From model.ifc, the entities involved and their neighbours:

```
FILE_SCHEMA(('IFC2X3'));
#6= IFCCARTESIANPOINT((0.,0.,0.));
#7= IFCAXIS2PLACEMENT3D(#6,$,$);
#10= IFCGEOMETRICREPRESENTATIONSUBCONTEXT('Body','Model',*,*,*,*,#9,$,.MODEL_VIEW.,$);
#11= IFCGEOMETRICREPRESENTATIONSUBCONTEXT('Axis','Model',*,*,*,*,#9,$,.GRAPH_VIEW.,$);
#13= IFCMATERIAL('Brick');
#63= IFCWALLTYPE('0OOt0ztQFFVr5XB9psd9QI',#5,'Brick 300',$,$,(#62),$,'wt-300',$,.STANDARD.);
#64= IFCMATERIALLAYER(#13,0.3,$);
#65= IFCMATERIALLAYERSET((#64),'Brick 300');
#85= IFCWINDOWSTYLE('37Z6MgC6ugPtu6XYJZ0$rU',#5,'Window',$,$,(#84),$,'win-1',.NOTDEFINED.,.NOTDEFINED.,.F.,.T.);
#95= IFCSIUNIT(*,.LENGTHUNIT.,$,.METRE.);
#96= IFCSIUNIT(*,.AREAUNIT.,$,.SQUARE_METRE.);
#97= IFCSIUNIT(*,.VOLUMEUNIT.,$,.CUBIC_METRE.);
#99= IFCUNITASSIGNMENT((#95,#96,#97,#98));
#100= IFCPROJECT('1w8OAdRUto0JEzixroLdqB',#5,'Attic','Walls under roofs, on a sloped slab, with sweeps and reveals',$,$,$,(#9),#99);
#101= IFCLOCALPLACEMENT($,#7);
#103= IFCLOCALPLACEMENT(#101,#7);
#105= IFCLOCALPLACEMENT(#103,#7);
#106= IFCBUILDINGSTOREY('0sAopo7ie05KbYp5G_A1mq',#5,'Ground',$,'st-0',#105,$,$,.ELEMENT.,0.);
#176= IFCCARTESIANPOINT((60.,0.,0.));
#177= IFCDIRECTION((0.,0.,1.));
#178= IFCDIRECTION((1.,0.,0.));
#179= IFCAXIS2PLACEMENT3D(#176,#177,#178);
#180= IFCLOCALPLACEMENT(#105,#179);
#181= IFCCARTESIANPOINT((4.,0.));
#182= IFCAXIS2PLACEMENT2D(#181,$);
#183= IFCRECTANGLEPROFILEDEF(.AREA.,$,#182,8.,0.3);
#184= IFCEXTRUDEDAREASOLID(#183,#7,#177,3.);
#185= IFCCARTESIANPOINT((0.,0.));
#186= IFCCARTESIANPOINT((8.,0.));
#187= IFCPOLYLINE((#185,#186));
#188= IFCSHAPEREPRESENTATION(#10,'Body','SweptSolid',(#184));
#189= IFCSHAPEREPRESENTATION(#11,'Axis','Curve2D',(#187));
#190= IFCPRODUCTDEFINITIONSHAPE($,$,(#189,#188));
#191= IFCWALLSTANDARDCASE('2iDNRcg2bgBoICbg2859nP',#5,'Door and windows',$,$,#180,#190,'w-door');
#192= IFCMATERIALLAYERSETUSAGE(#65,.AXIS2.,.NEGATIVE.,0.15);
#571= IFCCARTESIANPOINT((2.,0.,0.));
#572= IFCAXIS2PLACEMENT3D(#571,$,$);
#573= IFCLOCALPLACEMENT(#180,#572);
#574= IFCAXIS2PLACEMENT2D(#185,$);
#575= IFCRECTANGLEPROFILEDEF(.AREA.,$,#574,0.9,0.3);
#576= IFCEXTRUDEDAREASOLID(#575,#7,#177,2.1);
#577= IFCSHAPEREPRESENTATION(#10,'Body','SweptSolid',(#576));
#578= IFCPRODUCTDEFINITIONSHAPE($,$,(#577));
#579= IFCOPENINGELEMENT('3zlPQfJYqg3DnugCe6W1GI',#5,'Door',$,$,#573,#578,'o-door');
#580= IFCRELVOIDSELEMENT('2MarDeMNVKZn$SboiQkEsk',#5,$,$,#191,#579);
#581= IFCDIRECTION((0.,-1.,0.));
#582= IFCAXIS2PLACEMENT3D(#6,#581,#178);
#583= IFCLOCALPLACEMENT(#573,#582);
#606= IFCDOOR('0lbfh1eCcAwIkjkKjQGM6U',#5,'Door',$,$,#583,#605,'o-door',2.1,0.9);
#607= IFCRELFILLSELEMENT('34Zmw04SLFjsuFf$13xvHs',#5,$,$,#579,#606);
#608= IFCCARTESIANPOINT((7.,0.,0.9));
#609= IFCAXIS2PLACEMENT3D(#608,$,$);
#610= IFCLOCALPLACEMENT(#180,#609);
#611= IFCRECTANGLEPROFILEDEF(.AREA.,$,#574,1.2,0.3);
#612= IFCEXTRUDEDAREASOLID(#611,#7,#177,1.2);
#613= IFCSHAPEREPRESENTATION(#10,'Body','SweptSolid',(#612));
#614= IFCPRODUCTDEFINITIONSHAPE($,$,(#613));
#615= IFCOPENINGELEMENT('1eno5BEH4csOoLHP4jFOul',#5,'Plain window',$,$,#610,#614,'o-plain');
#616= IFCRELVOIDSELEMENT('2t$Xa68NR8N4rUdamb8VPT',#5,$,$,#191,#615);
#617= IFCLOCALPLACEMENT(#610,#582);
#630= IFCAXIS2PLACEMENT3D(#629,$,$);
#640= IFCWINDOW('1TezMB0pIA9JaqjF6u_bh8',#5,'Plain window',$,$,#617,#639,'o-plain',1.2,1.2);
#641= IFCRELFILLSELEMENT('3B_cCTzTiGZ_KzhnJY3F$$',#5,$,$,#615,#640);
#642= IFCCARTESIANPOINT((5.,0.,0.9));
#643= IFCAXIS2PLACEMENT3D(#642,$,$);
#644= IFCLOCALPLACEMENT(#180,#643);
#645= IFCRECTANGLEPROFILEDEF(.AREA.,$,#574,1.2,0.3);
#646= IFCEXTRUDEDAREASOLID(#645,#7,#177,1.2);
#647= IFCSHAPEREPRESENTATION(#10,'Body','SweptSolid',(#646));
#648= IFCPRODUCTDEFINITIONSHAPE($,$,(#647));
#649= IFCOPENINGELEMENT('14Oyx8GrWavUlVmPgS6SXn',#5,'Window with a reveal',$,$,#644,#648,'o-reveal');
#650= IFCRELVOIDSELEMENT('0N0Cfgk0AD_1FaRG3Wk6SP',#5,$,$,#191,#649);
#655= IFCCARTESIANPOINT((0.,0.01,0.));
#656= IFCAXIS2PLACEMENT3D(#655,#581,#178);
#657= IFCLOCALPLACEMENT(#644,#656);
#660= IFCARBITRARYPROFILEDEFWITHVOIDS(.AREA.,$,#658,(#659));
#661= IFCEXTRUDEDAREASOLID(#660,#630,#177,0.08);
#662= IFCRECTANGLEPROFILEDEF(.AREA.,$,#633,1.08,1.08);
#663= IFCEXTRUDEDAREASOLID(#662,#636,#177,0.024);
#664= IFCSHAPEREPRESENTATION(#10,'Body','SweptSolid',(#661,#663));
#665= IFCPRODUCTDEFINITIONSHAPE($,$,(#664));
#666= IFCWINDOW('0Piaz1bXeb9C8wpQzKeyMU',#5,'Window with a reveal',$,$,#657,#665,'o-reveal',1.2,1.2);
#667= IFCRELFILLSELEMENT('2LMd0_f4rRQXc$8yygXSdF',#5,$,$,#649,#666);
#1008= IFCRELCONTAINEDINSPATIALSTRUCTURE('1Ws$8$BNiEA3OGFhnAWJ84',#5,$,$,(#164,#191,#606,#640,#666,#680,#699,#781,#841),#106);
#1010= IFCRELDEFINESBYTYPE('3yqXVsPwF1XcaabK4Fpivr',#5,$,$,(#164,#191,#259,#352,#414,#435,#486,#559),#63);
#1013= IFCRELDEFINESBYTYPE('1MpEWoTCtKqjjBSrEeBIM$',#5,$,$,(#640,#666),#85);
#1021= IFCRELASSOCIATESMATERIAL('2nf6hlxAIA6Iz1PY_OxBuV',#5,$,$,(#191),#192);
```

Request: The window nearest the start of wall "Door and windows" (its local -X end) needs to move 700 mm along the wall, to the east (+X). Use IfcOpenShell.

```python
import ifcopenshell
import ifcopenshell.api.geometry
import ifcopenshell.util.placement

model = ifcopenshell.open("model.ifc")

window = model.by_guid("0Piaz1bXeb9C8wpQzKeyMU")
opening = window.FillsVoids[0].RelatingOpeningElement
wall = opening.VoidsElements[0].RelatingBuildingElement

wall_matrix = ifcopenshell.util.placement.get_local_placement(wall.ObjectPlacement)
shift = wall_matrix[:3, 0] * 0.7
before = ifcopenshell.util.placement.get_local_placement(window.ObjectPlacement)[:3, 3].copy()

# The window is placed relative to its opening, so it follows when the opening moves.
matrix = ifcopenshell.util.placement.get_local_placement(opening.ObjectPlacement)
matrix[:3, 3] += shift
ifcopenshell.api.geometry.edit_object_placement(
    model, product=opening, matrix=matrix, is_si=False, should_transform_children=True
)

after = ifcopenshell.util.placement.get_local_placement(window.ObjectPlacement)[:3, 3]
print("window moved by", (after - before).round(3) + 0.0)

model.write("model-out.ifc")
```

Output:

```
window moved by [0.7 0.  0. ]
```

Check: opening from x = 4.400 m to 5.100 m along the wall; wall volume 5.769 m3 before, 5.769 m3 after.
